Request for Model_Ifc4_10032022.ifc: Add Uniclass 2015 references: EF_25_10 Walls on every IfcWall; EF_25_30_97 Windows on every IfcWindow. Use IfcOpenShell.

First a look at what the model holds.

```python
import ifcopenshell

model = ifcopenshell.open("Model_Ifc4_10032022.ifc")
print(model.schema)
print("classifications:", [c.Name for c in model.by_type("IfcClassification")])
for ifc_class in ("IfcDoor", "IfcRoof", "IfcStair", "IfcWall", "IfcWindow"):
    print(ifc_class, len(model.by_type(ifc_class)))
```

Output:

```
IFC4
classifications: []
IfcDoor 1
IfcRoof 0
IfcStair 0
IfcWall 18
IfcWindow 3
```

```python
import ifcopenshell
import ifcopenshell.api.classification

model = ifcopenshell.open("Model_Ifc4_10032022.ifc")

system = ifcopenshell.api.classification.add_classification(model, classification="Uniclass 2015")

codes = {
    "IfcWall": ("EF_25_10", "Walls"),
    "IfcWindow": ("EF_25_30_97", "Windows"),
}
for ifc_class, (code, name) in codes.items():
    products = model.by_type(ifc_class)
    ifcopenshell.api.classification.add_reference(
        model, products=products, classification=system, identification=code, name=name
    )
    print(code, len(products))

model.write("Model_Ifc4_10032022_rev.ifc")
```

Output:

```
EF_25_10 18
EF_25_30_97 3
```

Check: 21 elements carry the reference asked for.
